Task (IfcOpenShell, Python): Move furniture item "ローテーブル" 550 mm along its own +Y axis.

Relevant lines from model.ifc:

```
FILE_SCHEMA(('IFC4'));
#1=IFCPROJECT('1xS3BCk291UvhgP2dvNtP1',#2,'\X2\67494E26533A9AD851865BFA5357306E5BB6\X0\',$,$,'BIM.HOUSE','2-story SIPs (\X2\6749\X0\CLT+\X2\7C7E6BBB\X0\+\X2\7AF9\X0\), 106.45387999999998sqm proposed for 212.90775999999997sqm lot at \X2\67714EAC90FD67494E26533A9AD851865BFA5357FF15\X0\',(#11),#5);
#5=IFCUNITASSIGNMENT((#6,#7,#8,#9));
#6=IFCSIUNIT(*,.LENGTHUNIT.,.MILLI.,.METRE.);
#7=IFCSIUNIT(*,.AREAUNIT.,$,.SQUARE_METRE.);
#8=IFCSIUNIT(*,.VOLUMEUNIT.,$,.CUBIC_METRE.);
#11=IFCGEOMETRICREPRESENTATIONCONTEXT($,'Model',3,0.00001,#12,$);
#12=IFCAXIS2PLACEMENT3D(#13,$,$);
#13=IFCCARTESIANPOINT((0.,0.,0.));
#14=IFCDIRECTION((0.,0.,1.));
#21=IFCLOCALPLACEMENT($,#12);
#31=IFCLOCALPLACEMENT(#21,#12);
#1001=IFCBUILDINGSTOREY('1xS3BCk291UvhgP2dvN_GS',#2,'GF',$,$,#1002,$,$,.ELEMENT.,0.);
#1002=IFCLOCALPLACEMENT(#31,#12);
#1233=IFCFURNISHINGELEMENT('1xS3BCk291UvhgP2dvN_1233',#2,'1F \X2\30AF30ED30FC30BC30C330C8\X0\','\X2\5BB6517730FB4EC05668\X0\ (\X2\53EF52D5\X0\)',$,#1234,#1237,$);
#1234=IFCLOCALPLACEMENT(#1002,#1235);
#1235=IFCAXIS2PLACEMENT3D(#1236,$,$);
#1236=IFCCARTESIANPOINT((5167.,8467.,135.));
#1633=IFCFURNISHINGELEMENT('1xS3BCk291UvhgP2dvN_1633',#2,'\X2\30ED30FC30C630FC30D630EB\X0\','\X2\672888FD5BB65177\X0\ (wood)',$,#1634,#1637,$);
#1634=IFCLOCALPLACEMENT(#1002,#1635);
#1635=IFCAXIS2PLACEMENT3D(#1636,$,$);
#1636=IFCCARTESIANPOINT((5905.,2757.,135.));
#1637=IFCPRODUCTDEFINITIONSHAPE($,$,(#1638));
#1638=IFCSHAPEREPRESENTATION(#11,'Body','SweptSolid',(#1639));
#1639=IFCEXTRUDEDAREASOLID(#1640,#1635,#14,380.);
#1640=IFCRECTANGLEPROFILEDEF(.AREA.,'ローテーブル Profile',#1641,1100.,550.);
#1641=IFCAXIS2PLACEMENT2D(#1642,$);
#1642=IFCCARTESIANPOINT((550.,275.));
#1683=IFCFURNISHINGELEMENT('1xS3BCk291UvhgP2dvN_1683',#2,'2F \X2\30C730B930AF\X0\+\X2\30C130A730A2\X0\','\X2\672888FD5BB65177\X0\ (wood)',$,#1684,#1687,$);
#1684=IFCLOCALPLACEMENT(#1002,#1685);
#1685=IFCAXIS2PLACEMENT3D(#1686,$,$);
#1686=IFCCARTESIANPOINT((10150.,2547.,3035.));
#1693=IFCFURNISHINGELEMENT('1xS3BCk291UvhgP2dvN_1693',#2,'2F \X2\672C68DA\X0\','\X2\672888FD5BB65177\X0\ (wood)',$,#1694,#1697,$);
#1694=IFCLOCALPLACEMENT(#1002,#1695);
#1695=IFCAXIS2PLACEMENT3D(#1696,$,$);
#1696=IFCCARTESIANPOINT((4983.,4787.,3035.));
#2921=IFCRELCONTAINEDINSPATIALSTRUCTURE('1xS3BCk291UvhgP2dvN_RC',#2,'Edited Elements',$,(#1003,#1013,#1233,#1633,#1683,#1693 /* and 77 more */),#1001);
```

```python
import ifcopenshell
import ifcopenshell.api.geometry
import ifcopenshell.util.placement

model = ifcopenshell.open("model.ifc")

item = model.by_id(1633)
matrix = ifcopenshell.util.placement.get_local_placement(item.ObjectPlacement)
matrix[:3, 3] += matrix[:3, 1] * 550.0
ifcopenshell.api.geometry.edit_object_placement(model, product=item, matrix=matrix, is_si=False)

print(ifcopenshell.util.placement.get_local_placement(item.ObjectPlacement).round(3) + 0.0)

model.write("model_updated.ifc")
```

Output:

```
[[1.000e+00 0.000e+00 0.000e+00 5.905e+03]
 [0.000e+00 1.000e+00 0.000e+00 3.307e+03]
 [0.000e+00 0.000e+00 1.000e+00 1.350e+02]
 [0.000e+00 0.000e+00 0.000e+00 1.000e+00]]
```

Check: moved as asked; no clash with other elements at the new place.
